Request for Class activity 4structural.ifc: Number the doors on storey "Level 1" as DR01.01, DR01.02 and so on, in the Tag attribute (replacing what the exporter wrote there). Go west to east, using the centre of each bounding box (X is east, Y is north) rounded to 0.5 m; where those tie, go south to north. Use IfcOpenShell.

First a look at what the model holds.

```python
import ifcopenshell
import ifcopenshell.util.element
import ifcopenshell.util.placement

model = ifcopenshell.open("Class activity 4structural.ifc")
print(model.schema)
storey = next(s for s in model.by_type("IfcBuildingStorey") if s.Name == "Level 1")
doors = [e for e in ifcopenshell.util.element.get_decomposition(storey) if e.is_a("IfcDoor")]
for e in sorted(doors, key=lambda e: e.id()):
    origin = ifcopenshell.util.placement.get_local_placement(e.ObjectPlacement)[:3, 3]
    print(e.id(), e.Tag, e.Name, origin.round(2) + 0.0, sep=" | ")
```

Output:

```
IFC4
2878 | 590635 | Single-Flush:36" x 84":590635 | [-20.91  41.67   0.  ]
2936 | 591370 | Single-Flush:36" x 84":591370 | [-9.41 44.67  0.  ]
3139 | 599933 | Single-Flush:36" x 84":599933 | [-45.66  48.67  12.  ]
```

```python
import ifcopenshell
import ifcopenshell.geom
import ifcopenshell.util.element
import ifcopenshell.util.shape

model = ifcopenshell.open("Class activity 4structural.ifc")
settings = ifcopenshell.geom.settings()
settings.set("use-world-coords", True)


def centre(element):
    shape = ifcopenshell.geom.create_shape(settings, element)
    return ifcopenshell.util.shape.get_bbox_centroid(shape.geometry)


storey = next(s for s in model.by_type("IfcBuildingStorey") if s.Name == "Level 1")
doors = [e for e in ifcopenshell.util.element.get_decomposition(storey) if e.is_a("IfcDoor")]

# Insertion points can sit at a corner or the storey origin, so sort by the geometry (in metres).
centres = {e: centre(e) for e in doors}
doors.sort(key=lambda e: (round(centres[e][0] / 0.5), centres[e][1]))

for i, e in enumerate(doors, start=1):
    number = f"DR01.{i:02d}"
    e.Tag = number
    print(e.id(), number)

model.write("Class activity 4structural-out.ifc")
```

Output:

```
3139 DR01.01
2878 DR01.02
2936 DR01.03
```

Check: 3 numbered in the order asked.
